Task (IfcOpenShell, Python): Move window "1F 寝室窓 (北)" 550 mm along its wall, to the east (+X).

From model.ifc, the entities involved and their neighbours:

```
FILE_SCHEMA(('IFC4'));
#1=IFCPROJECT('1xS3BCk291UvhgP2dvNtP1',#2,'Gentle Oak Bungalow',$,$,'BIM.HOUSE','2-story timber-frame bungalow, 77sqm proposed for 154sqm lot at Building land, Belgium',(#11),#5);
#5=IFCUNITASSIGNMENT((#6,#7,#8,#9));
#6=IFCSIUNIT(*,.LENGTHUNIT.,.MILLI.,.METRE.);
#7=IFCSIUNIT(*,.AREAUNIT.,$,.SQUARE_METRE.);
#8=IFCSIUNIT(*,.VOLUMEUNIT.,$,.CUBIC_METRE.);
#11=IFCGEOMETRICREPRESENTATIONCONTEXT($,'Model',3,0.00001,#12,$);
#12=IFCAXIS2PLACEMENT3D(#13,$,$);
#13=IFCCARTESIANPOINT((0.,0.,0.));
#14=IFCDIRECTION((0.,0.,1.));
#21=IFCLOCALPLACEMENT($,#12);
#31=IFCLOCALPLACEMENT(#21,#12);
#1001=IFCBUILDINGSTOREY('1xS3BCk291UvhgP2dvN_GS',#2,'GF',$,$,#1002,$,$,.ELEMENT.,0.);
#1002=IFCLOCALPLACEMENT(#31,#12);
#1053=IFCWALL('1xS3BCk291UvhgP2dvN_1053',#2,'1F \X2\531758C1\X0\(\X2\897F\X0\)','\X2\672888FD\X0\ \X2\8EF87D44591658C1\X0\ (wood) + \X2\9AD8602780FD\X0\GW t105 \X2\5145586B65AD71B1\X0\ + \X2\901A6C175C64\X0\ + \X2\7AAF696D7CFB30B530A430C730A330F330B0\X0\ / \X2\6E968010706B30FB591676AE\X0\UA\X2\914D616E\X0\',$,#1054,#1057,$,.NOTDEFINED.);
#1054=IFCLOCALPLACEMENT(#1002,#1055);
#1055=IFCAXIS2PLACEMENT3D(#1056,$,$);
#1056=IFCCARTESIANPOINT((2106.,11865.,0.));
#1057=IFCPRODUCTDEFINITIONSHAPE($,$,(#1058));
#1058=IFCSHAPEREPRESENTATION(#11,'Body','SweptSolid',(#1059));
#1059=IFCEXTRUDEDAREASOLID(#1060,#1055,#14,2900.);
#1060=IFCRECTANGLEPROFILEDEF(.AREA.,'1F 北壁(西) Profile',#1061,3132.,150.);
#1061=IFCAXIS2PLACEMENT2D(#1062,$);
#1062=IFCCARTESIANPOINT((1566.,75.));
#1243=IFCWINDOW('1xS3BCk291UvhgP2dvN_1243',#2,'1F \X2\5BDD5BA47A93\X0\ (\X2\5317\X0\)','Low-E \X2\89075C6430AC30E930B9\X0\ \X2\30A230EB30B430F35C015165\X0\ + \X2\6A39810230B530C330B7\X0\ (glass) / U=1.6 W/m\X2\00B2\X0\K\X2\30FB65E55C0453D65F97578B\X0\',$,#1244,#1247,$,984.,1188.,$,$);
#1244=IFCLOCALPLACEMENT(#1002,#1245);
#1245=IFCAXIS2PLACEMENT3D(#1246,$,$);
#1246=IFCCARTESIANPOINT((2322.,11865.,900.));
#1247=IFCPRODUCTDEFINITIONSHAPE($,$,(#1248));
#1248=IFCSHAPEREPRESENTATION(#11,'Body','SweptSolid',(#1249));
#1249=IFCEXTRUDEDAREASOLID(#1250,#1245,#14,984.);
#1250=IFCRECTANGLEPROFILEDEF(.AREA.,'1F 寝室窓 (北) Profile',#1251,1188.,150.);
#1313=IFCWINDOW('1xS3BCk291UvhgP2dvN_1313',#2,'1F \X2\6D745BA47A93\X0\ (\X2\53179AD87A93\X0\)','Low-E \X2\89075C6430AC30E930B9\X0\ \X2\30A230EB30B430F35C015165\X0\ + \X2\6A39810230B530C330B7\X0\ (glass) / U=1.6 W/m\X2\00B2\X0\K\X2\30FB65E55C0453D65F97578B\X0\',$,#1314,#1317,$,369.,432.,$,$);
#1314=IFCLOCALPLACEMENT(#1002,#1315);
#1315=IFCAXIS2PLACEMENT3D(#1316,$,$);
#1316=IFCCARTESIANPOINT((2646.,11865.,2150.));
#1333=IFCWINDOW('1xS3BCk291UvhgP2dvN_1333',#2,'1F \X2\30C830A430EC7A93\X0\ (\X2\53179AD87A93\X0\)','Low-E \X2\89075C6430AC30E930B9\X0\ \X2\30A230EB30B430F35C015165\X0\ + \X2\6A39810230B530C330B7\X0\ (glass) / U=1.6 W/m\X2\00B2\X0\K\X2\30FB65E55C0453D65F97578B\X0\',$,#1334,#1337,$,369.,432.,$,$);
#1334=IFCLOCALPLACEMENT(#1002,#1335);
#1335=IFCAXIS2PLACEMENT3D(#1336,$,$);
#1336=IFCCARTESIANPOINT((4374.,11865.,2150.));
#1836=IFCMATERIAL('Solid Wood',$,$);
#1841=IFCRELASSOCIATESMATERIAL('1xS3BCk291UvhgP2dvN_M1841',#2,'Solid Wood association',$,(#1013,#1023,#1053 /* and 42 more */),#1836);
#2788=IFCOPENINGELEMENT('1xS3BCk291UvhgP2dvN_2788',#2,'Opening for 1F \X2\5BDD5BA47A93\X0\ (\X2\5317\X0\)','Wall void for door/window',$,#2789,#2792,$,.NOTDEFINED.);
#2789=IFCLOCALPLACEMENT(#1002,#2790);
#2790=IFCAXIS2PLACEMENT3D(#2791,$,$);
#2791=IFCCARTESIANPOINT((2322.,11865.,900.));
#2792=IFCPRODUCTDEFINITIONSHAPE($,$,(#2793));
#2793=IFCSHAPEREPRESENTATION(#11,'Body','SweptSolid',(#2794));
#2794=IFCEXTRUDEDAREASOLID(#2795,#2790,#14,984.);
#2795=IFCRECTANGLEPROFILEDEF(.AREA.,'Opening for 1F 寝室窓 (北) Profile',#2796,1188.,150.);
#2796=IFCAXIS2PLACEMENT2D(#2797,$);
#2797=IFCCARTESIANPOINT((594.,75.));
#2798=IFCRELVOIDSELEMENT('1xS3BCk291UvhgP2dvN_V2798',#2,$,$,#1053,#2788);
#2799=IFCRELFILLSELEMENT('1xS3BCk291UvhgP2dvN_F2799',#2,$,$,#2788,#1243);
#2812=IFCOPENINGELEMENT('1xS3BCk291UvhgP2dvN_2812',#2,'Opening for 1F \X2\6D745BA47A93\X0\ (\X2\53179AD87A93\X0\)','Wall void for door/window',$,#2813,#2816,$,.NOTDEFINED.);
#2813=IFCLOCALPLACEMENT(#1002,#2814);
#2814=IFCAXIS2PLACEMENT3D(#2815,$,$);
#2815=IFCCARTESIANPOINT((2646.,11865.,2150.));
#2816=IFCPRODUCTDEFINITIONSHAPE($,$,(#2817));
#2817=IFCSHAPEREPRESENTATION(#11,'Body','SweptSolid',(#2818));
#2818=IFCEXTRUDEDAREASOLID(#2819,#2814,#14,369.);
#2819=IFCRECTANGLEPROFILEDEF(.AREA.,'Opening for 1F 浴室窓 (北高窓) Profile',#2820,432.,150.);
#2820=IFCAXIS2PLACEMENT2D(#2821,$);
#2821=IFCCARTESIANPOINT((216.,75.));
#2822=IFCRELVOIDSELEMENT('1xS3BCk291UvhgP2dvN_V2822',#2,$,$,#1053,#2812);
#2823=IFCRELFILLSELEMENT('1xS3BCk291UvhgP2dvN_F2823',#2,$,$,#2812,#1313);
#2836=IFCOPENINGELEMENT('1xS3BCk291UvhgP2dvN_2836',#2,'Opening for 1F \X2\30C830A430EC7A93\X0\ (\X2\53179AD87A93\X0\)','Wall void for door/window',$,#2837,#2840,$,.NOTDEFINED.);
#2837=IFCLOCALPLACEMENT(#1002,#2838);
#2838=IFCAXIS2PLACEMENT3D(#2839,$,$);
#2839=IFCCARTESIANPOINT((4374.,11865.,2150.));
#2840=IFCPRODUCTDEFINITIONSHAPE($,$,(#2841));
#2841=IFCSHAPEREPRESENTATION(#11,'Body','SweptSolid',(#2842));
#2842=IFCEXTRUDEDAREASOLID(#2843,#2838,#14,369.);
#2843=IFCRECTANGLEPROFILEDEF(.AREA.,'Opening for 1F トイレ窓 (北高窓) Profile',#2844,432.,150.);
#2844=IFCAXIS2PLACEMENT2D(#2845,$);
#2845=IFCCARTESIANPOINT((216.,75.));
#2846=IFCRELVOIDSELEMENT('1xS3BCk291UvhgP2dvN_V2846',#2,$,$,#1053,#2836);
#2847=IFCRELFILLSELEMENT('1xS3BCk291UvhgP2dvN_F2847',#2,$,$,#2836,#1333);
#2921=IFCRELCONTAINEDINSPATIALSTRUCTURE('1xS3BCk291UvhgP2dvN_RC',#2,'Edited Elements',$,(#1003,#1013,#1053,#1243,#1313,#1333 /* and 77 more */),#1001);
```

```python
import ifcopenshell
import ifcopenshell.api.geometry
import ifcopenshell.util.placement

model = ifcopenshell.open("model.ifc")

window = model.by_guid("1xS3BCk291UvhgP2dvN_1243")
opening = window.FillsVoids[0].RelatingOpeningElement
wall = opening.VoidsElements[0].RelatingBuildingElement

wall_matrix = ifcopenshell.util.placement.get_local_placement(wall.ObjectPlacement)
shift = wall_matrix[:3, 0] * 550.0
before = ifcopenshell.util.placement.get_local_placement(window.ObjectPlacement)[:3, 3].copy()

# The window is not placed relative to its opening, so move both.
for product in (opening, window):
    matrix = ifcopenshell.util.placement.get_local_placement(product.ObjectPlacement)
    matrix[:3, 3] += shift
    ifcopenshell.api.geometry.edit_object_placement(model, product=product, matrix=matrix, is_si=False)

after = ifcopenshell.util.placement.get_local_placement(window.ObjectPlacement)[:3, 3]
print("window moved by", (after - before).round(3) + 0.0)

model.write("model_updated.ifc")
```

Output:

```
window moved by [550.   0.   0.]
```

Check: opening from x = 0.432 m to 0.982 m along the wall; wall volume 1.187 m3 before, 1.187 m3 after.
